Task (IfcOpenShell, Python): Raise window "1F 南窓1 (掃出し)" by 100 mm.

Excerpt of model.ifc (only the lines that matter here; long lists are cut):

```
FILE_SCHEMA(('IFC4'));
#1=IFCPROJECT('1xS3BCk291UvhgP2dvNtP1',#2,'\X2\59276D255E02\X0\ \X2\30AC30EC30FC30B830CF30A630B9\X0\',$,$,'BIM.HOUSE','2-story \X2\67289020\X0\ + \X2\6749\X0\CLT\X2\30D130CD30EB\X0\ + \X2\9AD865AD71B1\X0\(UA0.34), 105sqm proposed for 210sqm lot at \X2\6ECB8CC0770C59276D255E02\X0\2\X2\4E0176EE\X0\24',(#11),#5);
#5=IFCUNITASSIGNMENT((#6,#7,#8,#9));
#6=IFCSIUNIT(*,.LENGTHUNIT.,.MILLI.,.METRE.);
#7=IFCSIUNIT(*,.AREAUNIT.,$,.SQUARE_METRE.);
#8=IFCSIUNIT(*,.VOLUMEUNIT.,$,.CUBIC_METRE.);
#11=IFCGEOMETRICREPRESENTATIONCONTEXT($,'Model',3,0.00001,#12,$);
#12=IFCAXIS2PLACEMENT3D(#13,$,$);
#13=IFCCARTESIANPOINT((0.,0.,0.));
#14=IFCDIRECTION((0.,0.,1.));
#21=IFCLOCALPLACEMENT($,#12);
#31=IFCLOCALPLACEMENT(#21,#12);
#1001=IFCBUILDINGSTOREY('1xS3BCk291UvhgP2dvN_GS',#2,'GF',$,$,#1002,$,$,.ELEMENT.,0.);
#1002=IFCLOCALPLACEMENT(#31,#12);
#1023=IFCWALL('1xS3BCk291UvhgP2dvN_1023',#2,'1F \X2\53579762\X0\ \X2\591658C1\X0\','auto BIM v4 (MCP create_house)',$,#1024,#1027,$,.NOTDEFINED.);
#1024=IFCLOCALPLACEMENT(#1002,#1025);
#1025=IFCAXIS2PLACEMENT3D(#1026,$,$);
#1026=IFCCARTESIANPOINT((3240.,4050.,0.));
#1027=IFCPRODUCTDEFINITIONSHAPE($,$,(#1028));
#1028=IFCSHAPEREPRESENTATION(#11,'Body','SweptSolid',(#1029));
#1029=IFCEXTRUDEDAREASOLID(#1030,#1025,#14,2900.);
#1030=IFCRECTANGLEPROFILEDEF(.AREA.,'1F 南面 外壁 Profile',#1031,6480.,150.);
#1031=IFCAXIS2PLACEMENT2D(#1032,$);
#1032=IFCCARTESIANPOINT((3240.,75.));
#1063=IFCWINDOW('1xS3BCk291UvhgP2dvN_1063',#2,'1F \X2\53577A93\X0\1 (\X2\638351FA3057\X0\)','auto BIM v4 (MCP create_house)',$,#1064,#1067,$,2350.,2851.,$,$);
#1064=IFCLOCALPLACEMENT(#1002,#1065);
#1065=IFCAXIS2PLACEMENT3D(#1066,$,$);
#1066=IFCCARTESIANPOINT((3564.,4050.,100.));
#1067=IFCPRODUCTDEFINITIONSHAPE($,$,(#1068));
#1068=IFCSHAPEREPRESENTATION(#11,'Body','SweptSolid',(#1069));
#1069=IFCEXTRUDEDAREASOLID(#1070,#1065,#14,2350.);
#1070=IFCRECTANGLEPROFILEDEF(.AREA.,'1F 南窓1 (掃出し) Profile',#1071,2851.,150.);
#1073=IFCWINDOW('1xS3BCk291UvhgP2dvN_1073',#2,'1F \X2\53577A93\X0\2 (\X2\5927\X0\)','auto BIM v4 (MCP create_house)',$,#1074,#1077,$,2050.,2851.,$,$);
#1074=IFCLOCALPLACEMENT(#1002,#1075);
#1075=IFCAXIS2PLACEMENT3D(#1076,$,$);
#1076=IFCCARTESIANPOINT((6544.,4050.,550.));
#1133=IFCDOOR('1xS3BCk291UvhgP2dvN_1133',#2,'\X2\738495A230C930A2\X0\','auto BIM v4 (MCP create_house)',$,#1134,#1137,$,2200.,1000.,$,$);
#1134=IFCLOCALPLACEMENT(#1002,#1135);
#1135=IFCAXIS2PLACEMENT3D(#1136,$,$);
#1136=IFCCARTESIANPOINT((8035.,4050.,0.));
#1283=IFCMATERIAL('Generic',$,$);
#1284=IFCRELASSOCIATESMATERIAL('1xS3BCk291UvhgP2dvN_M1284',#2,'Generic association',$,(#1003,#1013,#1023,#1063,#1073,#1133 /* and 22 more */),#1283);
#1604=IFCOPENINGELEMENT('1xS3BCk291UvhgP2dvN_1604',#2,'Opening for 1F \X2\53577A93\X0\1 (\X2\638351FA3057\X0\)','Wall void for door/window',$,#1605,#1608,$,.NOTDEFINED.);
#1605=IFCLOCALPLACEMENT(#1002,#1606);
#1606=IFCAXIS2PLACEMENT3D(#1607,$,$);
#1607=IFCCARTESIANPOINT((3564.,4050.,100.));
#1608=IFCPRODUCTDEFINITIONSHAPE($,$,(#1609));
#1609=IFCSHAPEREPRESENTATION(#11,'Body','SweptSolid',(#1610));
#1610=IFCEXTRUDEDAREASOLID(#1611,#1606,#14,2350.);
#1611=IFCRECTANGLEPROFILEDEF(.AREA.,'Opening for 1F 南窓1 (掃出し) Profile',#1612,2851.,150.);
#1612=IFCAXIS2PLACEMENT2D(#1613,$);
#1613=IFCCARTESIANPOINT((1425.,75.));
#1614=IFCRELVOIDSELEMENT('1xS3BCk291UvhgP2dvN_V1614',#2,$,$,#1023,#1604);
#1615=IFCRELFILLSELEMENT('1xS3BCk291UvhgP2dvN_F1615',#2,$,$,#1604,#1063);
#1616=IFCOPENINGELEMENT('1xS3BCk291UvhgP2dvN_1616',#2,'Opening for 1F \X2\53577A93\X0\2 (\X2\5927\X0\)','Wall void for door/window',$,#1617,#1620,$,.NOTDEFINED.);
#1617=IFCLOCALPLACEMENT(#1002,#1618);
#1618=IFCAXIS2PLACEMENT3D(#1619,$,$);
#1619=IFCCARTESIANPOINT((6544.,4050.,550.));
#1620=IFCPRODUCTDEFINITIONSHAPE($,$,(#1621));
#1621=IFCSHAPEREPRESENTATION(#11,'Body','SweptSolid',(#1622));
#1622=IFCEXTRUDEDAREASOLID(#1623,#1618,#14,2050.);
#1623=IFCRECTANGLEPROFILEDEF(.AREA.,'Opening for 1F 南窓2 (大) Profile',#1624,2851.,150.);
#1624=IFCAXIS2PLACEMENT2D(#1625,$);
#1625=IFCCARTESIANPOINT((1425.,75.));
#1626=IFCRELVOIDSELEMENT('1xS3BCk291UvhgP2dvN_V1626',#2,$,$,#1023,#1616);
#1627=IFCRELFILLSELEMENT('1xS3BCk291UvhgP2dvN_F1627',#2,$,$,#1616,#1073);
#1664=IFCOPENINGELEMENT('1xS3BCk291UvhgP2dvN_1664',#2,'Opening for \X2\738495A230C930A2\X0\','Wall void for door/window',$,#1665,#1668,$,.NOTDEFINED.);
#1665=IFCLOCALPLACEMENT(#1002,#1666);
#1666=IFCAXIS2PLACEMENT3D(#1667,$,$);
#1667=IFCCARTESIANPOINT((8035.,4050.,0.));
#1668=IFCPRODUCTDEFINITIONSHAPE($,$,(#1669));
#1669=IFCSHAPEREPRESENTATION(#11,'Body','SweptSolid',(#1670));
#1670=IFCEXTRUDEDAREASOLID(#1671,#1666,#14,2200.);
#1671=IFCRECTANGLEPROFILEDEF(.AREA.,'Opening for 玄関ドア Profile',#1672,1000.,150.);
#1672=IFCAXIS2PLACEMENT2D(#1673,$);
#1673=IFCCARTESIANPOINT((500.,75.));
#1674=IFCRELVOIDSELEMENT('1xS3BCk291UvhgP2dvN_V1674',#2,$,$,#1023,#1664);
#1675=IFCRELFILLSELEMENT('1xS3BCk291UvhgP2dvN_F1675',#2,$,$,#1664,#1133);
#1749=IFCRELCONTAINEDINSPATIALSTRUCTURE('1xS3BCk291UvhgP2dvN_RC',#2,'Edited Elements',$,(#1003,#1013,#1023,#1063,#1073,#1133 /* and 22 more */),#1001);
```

```python
import numpy as np
import ifcopenshell
import ifcopenshell.api.geometry
import ifcopenshell.util.placement
import ifcopenshell.util.unit

model = ifcopenshell.open("model.ifc")
unit_scale = ifcopenshell.util.unit.calculate_unit_scale(model)

window = model.by_guid("1xS3BCk291UvhgP2dvN_1063")
opening = window.FillsVoids[0].RelatingOpeningElement
dz = 100.0

shift = np.array([0.0, 0.0, dz])
# The window is not placed relative to its opening, so move both.
for product in (opening, window):
    matrix = ifcopenshell.util.placement.get_local_placement(product.ObjectPlacement)
    matrix[:3, 3] += shift
    ifcopenshell.api.geometry.edit_object_placement(model, product=product, matrix=matrix, is_si=False)

print(f"moved by {dz * unit_scale:+.3f} m")

model.write("model_rev.ifc")
```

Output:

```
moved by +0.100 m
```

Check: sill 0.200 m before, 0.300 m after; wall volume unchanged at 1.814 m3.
